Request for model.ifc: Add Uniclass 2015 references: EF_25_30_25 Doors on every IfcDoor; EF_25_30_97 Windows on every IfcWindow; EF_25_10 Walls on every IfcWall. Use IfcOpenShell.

First a look at what the model holds.

```python
import ifcopenshell

model = ifcopenshell.open("model.ifc")
print(model.schema)
print("classifications:", [c.Name for c in model.by_type("IfcClassification")])
for ifc_class in ("IfcDoor", "IfcRoof", "IfcStair", "IfcWall", "IfcWindow"):
    print(ifc_class, len(model.by_type(ifc_class)))
```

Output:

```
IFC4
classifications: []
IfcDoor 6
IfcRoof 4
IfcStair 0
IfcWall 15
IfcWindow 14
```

```python
import ifcopenshell
import ifcopenshell.api.classification

model = ifcopenshell.open("model.ifc")

system = ifcopenshell.api.classification.add_classification(model, classification="Uniclass 2015")

codes = {
    "IfcDoor": ("EF_25_30_25", "Doors"),
    "IfcWindow": ("EF_25_30_97", "Windows"),
    "IfcWall": ("EF_25_10", "Walls"),
}
for ifc_class, (code, name) in codes.items():
    products = model.by_type(ifc_class)
    ifcopenshell.api.classification.add_reference(
        model, products=products, classification=system, identification=code, name=name
    )
    print(code, len(products))

model.write("model_updated.ifc")
```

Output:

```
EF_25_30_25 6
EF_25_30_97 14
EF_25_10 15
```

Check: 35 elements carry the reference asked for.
